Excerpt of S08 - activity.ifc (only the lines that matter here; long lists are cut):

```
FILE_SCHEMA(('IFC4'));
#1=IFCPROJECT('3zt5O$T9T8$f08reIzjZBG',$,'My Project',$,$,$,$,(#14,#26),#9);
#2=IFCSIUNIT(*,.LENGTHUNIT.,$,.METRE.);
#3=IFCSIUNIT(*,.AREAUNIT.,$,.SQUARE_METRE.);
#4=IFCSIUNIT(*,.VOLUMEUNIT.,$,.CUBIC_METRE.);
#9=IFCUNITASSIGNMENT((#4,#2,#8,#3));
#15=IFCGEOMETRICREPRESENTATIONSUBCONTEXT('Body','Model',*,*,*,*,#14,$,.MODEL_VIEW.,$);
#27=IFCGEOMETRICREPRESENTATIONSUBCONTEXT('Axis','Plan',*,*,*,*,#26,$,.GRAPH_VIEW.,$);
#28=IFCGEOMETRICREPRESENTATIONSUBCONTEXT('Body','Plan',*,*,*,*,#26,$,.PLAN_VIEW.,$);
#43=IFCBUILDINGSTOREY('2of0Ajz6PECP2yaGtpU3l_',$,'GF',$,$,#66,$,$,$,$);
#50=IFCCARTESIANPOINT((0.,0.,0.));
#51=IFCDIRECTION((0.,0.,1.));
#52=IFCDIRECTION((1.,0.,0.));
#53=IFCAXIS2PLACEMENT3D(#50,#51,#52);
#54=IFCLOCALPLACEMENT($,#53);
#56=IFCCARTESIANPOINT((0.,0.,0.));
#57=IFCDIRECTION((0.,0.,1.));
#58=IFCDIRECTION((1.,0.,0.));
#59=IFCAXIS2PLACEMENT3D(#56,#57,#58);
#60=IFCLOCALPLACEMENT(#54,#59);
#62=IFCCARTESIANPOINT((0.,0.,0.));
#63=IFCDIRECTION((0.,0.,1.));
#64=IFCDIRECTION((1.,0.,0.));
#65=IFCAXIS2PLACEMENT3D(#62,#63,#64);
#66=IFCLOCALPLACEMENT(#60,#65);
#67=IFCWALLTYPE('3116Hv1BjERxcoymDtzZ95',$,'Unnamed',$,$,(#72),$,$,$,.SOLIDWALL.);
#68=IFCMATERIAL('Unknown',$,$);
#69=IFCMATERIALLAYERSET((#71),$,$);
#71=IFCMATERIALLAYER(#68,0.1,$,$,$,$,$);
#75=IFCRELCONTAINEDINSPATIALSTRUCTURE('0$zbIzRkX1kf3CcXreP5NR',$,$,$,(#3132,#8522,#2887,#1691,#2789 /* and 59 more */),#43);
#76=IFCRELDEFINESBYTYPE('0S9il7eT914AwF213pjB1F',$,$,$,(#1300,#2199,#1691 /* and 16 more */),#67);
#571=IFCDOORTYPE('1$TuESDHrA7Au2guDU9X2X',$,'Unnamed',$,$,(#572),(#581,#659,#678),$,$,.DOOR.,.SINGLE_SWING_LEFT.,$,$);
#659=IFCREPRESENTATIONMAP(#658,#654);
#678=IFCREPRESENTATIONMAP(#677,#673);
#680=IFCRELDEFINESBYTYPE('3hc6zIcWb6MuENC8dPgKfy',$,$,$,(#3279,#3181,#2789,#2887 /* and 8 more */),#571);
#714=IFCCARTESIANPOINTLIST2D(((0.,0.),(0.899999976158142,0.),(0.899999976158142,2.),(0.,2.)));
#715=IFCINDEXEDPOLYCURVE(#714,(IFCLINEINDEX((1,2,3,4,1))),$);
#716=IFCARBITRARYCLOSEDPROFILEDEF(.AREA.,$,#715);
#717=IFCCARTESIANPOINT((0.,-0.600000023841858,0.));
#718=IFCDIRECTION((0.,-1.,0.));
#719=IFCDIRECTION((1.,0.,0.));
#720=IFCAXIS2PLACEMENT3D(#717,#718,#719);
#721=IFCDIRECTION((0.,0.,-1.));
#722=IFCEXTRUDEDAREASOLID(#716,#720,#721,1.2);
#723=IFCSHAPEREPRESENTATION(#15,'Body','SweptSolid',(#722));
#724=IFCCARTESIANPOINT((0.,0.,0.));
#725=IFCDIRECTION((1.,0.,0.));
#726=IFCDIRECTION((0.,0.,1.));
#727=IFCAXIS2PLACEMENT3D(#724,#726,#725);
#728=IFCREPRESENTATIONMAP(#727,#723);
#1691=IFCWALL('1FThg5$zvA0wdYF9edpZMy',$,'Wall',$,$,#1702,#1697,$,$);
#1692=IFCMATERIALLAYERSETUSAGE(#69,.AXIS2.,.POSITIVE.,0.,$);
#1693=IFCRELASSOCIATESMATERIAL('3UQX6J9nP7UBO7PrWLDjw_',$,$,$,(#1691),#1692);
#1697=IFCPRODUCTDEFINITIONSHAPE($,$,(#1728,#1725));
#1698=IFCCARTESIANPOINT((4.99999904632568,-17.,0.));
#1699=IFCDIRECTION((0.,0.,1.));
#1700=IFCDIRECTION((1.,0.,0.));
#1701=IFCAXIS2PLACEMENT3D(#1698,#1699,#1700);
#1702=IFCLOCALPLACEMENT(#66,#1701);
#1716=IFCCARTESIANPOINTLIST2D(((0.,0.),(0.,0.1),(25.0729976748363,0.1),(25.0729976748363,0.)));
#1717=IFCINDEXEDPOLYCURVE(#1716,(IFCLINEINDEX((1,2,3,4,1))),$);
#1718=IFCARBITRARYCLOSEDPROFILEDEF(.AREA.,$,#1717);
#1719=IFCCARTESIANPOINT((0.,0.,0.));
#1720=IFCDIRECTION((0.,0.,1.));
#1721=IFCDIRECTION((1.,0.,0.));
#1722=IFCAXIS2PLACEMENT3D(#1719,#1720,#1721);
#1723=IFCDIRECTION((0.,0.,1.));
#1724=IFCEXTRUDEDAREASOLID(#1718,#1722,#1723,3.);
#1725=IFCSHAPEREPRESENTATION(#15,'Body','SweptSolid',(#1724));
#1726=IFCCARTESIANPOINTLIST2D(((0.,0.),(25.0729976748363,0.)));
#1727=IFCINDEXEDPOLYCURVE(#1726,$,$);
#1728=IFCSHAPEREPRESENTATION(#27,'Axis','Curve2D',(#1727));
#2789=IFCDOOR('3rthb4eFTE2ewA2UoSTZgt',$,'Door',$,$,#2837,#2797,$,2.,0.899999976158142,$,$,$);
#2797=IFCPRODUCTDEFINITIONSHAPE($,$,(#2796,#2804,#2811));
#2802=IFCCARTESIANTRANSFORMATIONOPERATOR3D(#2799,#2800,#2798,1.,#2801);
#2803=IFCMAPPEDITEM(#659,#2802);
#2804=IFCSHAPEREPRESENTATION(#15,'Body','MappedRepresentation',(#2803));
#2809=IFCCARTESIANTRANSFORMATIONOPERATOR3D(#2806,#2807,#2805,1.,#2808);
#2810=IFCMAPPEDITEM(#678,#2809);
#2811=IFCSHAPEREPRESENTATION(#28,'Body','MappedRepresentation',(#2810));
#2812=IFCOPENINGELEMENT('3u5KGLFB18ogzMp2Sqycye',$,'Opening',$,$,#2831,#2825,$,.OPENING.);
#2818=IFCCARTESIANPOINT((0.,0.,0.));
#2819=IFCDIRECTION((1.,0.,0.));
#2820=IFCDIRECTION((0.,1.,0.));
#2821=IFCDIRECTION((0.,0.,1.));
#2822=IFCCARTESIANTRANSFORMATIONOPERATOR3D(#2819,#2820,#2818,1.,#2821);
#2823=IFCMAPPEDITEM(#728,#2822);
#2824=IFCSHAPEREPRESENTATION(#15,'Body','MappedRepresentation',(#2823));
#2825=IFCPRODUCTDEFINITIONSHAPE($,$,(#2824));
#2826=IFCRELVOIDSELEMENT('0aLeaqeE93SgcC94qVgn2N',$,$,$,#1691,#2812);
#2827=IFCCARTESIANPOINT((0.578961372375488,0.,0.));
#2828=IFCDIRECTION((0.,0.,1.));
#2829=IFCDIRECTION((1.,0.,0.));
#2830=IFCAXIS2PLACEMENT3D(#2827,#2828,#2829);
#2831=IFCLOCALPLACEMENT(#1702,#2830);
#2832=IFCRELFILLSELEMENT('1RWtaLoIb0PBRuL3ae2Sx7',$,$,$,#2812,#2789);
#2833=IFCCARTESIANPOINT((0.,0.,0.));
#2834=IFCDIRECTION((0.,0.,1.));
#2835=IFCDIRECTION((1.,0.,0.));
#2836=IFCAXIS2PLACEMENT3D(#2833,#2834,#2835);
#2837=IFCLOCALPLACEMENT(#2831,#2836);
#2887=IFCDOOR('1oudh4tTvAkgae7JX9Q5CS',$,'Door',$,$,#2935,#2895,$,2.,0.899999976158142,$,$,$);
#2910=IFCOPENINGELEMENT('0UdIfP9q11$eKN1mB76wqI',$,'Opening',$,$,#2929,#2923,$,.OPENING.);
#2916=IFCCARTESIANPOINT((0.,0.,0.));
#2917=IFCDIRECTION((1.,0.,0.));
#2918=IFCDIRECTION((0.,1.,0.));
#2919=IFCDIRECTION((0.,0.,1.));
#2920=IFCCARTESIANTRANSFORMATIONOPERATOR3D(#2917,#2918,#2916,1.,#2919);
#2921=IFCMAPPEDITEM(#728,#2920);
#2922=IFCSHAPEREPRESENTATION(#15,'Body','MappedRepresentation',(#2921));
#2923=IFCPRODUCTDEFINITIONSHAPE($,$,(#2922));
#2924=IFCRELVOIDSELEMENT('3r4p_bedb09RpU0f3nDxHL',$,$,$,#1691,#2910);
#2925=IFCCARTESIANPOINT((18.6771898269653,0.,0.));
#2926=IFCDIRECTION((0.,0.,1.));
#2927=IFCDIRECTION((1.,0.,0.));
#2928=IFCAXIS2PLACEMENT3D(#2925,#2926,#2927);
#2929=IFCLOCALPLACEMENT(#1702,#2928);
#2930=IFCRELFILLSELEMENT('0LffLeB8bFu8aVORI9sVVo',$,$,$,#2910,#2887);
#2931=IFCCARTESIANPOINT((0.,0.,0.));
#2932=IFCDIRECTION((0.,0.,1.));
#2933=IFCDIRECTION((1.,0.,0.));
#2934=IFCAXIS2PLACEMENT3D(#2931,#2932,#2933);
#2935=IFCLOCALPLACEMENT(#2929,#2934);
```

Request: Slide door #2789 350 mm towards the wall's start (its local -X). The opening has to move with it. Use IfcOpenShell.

```python
import ifcopenshell
import ifcopenshell.api.geometry
import ifcopenshell.util.placement
import ifcopenshell.util.unit

model = ifcopenshell.open("S08 - activity.ifc")
unit_scale = ifcopenshell.util.unit.calculate_unit_scale(model)

door = model.by_guid("3rthb4eFTE2ewA2UoSTZgt")
opening = door.FillsVoids[0].RelatingOpeningElement
wall = opening.VoidsElements[0].RelatingBuildingElement

wall_matrix = ifcopenshell.util.placement.get_local_placement(wall.ObjectPlacement)
shift = wall_matrix[:3, 0] * -0.35 / unit_scale
before = ifcopenshell.util.placement.get_local_placement(door.ObjectPlacement)[:3, 3].copy()

# The door is placed relative to its opening, so it follows when the opening moves.
matrix = ifcopenshell.util.placement.get_local_placement(opening.ObjectPlacement)
matrix[:3, 3] += shift
ifcopenshell.api.geometry.edit_object_placement(
    model, product=opening, matrix=matrix, is_si=False, should_transform_children=True
)

after = ifcopenshell.util.placement.get_local_placement(door.ObjectPlacement)[:3, 3]
print("door moved by", (after - before).round(3) + 0.0)

model.write("S08 - activity_rev.ifc")
```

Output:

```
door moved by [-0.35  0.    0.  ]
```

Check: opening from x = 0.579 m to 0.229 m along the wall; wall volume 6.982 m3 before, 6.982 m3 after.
